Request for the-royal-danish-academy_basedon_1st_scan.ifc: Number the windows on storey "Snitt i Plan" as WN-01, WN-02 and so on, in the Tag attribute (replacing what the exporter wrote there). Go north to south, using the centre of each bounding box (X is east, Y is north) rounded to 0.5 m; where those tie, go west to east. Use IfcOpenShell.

First a look at what the model holds.

```python
import ifcopenshell
import ifcopenshell.util.element
import ifcopenshell.util.placement

model = ifcopenshell.open("the-royal-danish-academy_basedon_1st_scan.ifc")
print(model.schema)
storey = next(s for s in model.by_type("IfcBuildingStorey") if s.Name == "Snitt i Plan")
windows = [e for e in ifcopenshell.util.element.get_decomposition(storey) if e.is_a("IfcWindow")]
for e in sorted(windows, key=lambda e: e.id()):
    origin = ifcopenshell.util.placement.get_local_placement(e.ObjectPlacement)[:3, 3]
    print(e.id(), e.Tag, e.Name, origin.round(2) + 0.0, sep=" | ")
```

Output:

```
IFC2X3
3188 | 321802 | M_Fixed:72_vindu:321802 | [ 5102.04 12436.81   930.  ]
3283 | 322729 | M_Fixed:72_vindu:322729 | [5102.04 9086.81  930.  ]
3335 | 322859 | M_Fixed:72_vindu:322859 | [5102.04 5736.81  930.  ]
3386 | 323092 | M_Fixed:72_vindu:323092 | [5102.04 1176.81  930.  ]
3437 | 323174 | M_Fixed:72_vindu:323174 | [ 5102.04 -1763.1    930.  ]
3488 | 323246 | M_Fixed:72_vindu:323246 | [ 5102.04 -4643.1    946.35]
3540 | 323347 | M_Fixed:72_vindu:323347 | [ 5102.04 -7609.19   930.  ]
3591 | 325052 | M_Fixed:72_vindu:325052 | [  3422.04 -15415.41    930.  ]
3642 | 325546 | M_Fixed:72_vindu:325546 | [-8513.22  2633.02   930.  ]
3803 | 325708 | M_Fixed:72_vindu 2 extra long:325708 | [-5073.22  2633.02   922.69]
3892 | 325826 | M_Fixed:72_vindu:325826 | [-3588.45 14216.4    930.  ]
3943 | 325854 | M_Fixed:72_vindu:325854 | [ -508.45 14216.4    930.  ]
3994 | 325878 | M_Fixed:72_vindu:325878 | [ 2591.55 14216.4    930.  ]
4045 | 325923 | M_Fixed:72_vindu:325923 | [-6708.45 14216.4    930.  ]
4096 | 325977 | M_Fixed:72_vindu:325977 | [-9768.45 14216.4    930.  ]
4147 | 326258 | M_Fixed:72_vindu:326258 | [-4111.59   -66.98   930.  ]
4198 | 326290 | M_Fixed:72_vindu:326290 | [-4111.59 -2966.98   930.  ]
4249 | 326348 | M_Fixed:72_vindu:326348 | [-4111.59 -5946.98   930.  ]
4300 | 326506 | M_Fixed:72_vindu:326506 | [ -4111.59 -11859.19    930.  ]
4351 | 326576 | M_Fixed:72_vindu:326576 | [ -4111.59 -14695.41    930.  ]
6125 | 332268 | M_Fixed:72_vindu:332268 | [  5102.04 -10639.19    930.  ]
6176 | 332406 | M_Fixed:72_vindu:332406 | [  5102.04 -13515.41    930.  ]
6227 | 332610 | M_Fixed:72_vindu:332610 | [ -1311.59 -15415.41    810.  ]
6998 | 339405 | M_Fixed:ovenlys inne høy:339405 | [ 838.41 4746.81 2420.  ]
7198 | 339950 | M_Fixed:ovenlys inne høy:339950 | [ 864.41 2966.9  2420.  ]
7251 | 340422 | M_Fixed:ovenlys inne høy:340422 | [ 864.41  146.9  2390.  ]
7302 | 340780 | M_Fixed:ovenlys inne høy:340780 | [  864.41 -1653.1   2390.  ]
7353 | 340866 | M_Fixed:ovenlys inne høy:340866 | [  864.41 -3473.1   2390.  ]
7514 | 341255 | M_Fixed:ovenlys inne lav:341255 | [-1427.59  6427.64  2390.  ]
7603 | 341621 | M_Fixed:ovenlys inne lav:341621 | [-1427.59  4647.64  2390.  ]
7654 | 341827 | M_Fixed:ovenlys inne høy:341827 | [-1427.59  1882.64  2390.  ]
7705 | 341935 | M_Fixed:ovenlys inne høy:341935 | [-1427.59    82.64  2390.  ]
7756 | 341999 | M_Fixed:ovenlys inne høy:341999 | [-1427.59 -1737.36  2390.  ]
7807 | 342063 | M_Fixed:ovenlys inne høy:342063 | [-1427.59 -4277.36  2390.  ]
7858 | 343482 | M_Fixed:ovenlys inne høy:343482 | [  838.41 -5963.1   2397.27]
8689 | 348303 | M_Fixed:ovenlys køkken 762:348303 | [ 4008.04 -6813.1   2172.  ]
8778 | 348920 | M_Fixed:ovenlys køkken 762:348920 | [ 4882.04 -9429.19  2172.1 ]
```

```python
import ifcopenshell
import ifcopenshell.geom
import ifcopenshell.util.element
import ifcopenshell.util.shape

model = ifcopenshell.open("the-royal-danish-academy_basedon_1st_scan.ifc")
settings = ifcopenshell.geom.settings()
settings.set("use-world-coords", True)


def centre(element):
    shape = ifcopenshell.geom.create_shape(settings, element)
    return ifcopenshell.util.shape.get_bbox_centroid(shape.geometry)


storey = next(s for s in model.by_type("IfcBuildingStorey") if s.Name == "Snitt i Plan")
windows = [e for e in ifcopenshell.util.element.get_decomposition(storey) if e.is_a("IfcWindow")]

# Insertion points can sit at a corner or the storey origin, so sort by the geometry (in metres).
centres = {e: centre(e) for e in windows}
windows.sort(key=lambda e: (-round(centres[e][1] / 0.5), centres[e][0]))

for i, e in enumerate(windows, start=1):
    number = f"WN-{i:02d}"
    e.Tag = number
    print(e.id(), number)

model.write("the-royal-danish-academy_basedon_1st_scan_rev.ifc")
```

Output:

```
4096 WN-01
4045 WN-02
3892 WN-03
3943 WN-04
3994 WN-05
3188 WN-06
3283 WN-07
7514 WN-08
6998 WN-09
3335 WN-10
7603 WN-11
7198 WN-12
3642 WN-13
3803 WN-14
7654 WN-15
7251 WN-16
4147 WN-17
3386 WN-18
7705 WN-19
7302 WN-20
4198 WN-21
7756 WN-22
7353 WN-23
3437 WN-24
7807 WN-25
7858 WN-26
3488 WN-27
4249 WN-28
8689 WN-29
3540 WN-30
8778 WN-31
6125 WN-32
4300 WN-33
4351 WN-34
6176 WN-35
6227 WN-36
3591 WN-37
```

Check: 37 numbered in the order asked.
